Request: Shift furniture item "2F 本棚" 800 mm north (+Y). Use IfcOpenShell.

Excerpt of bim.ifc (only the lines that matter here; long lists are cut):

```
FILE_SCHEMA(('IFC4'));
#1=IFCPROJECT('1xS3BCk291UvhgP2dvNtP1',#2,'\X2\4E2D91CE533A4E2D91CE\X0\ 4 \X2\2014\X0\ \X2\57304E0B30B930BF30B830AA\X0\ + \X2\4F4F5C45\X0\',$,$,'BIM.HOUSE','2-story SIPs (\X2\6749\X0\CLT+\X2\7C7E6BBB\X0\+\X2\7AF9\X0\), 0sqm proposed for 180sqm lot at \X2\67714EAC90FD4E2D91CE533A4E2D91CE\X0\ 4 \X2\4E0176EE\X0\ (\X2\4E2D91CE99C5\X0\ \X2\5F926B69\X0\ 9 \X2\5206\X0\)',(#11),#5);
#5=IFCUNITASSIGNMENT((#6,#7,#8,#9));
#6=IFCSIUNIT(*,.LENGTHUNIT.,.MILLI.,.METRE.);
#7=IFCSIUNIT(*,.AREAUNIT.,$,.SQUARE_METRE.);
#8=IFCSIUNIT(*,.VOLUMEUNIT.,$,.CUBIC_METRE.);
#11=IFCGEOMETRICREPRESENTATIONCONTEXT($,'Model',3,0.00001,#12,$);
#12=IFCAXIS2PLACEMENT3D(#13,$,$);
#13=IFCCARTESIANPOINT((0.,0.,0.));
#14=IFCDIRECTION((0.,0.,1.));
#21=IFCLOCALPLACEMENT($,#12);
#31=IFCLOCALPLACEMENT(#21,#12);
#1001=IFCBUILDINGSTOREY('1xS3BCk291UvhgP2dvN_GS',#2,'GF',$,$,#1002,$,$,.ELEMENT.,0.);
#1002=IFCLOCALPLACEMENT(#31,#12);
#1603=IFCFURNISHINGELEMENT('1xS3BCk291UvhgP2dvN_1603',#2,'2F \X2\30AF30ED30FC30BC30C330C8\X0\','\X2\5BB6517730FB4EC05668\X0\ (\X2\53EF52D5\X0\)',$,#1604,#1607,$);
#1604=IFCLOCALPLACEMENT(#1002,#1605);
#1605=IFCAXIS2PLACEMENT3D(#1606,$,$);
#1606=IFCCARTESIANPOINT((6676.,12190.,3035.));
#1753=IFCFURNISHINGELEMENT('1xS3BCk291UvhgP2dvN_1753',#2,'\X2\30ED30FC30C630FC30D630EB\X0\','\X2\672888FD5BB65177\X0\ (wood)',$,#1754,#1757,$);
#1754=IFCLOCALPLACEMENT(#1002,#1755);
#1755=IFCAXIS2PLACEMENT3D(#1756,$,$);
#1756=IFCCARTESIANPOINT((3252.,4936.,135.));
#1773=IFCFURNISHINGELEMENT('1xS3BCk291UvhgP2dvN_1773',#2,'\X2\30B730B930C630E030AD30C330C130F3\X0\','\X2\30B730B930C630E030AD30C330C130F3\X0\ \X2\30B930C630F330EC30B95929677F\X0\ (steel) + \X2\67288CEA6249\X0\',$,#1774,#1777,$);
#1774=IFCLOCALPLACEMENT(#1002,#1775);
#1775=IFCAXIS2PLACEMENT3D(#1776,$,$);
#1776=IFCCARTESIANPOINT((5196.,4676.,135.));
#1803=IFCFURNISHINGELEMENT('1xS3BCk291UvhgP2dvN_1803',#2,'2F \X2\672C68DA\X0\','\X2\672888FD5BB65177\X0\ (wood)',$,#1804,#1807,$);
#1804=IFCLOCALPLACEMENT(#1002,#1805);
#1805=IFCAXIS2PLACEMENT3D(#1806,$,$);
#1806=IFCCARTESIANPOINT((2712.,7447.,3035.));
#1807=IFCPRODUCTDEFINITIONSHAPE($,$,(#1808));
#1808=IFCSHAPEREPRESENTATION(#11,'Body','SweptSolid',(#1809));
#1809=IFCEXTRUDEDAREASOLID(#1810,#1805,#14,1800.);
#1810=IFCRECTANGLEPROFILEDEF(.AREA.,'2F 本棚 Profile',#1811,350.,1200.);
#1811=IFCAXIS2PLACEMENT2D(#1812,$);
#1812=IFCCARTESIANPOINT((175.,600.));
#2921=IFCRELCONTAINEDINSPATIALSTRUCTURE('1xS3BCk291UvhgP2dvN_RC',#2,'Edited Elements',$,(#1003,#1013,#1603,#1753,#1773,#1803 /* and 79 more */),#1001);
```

```python
import ifcopenshell
import ifcopenshell.api.geometry
import ifcopenshell.util.placement

model = ifcopenshell.open("bim.ifc")

item = model.by_guid("1xS3BCk291UvhgP2dvN_1803")
matrix = ifcopenshell.util.placement.get_local_placement(item.ObjectPlacement)
matrix[1, 3] += 800.0
ifcopenshell.api.geometry.edit_object_placement(model, product=item, matrix=matrix, is_si=False)

print(ifcopenshell.util.placement.get_local_placement(item.ObjectPlacement).round(3) + 0.0)

model.write("bim-out.ifc")
```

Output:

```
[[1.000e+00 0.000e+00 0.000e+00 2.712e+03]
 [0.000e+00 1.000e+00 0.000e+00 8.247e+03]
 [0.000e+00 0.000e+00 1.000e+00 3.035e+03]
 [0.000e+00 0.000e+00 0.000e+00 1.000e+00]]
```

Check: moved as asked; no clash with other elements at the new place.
